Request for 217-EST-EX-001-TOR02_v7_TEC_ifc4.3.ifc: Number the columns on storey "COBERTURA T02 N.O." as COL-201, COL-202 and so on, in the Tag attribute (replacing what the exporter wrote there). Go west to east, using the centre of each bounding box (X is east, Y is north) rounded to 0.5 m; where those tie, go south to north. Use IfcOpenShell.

First a look at what the model holds.

```python
import ifcopenshell
import ifcopenshell.util.element
import ifcopenshell.util.placement

model = ifcopenshell.open("217-EST-EX-001-TOR02_v7_TEC_ifc4.3.ifc")
print(model.schema)
storey = next(s for s in model.by_type("IfcBuildingStorey") if s.Name == "COBERTURA T02 N.O.")
columns = [e for e in ifcopenshell.util.element.get_decomposition(storey) if e.is_a("IfcColumn")]
for e in sorted(columns, key=lambda e: e.id()):
    origin = ifcopenshell.util.placement.get_local_placement(e.ObjectPlacement)[:3, 3]
    print(e.id(), e.Tag, e.Name, origin.round(2) + 0.0, sep=" | ")
```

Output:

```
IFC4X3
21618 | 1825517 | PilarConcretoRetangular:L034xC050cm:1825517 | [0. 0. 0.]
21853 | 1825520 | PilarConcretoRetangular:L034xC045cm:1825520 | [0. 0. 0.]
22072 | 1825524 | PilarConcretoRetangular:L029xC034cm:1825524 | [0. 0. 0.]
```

```python
import ifcopenshell
import ifcopenshell.geom
import ifcopenshell.util.element
import ifcopenshell.util.shape

model = ifcopenshell.open("217-EST-EX-001-TOR02_v7_TEC_ifc4.3.ifc")
settings = ifcopenshell.geom.settings()
settings.set("use-world-coords", True)


def centre(element):
    shape = ifcopenshell.geom.create_shape(settings, element)
    return ifcopenshell.util.shape.get_bbox_centroid(shape.geometry)


storey = next(s for s in model.by_type("IfcBuildingStorey") if s.Name == "COBERTURA T02 N.O.")
columns = [e for e in ifcopenshell.util.element.get_decomposition(storey) if e.is_a("IfcColumn")]

# Insertion points can sit at a corner or the storey origin, so sort by the geometry (in metres).
centres = {e: centre(e) for e in columns}
columns.sort(key=lambda e: (round(centres[e][0] / 0.5), centres[e][1]))

for i, e in enumerate(columns, start=1):
    number = f"COL-2{i:02d}"
    e.Tag = number
    print(e.id(), number)

model.write("217-EST-EX-001-TOR02_v7_TEC_ifc4.3_updated.ifc")
```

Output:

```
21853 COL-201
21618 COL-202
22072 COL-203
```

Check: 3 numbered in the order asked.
